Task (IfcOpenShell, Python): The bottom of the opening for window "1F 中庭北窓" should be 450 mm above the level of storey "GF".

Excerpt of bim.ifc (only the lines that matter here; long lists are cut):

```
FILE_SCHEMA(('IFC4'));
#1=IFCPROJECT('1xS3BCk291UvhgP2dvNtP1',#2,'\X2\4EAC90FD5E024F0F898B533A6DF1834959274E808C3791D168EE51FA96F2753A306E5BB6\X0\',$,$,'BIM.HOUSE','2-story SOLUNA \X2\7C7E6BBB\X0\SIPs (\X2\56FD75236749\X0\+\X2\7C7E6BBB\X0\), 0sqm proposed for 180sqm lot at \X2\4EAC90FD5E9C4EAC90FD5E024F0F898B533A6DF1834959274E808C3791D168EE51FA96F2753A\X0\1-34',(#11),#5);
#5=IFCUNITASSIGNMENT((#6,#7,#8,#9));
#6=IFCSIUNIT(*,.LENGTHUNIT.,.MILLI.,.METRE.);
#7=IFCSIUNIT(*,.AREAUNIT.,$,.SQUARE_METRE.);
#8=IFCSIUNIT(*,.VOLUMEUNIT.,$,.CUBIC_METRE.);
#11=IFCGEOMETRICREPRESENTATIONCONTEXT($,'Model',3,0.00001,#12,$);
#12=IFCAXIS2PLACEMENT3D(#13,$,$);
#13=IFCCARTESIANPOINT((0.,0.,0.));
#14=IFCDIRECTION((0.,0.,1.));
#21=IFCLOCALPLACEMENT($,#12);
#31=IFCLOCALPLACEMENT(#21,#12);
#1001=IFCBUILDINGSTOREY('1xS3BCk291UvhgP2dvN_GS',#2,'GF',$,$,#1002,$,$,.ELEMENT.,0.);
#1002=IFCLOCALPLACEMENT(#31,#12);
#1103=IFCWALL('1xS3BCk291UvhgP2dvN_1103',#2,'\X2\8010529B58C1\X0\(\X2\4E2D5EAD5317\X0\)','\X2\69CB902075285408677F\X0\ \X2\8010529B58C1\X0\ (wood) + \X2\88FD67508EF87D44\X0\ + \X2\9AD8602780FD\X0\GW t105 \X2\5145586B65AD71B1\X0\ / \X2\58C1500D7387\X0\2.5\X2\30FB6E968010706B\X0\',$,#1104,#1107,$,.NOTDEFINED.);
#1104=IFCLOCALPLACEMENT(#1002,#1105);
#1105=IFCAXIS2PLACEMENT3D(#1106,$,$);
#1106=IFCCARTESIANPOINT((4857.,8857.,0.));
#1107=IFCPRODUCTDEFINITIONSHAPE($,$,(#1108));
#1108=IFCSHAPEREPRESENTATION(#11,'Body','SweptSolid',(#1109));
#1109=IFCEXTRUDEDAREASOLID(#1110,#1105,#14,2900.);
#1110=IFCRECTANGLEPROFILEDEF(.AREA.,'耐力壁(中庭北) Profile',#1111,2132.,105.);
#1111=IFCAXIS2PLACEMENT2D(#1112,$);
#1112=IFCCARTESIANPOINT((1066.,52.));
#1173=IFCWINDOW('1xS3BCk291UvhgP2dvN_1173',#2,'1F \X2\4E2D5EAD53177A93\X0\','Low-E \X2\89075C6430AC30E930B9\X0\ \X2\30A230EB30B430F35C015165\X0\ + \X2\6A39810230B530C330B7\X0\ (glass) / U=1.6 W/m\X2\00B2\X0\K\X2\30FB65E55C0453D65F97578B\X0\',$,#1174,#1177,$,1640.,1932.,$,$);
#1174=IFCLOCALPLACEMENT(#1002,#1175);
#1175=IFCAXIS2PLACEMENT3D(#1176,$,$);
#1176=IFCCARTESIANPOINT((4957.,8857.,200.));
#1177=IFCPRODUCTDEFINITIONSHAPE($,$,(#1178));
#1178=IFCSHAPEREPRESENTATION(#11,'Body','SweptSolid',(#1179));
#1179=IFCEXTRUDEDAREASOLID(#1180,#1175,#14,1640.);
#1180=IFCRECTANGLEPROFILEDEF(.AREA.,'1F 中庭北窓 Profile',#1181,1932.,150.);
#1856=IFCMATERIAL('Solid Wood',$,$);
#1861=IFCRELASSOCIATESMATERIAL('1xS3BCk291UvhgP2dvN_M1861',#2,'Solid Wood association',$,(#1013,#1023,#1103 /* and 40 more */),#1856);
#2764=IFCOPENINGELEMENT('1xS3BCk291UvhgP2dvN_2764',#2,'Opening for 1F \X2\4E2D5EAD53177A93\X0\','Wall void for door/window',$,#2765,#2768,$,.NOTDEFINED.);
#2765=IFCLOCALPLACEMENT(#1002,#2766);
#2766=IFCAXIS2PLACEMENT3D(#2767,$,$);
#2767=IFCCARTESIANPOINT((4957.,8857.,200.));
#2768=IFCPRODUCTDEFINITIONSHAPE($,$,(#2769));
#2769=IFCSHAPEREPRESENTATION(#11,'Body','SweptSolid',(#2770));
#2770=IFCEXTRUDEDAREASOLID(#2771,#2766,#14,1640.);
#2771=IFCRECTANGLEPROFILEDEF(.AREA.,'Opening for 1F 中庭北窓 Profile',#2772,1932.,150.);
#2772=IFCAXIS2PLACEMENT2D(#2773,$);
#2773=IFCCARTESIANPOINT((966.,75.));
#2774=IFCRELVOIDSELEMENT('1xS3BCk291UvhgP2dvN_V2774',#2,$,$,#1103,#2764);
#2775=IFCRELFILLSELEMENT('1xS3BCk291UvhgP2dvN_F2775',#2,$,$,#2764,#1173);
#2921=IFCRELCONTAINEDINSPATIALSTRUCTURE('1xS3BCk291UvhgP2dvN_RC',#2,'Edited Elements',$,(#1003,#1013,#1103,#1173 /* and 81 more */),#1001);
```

```python
import numpy as np
import ifcopenshell
import ifcopenshell.api.geometry
import ifcopenshell.geom
import ifcopenshell.util.element
import ifcopenshell.util.placement
import ifcopenshell.util.shape
import ifcopenshell.util.unit

model = ifcopenshell.open("bim.ifc")
unit_scale = ifcopenshell.util.unit.calculate_unit_scale(model)

window = model.by_guid("1xS3BCk291UvhgP2dvN_1173")
opening = window.FillsVoids[0].RelatingOpeningElement
storey = ifcopenshell.util.element.get_container(window, ifc_class="IfcBuildingStorey")
level = ifcopenshell.util.placement.get_local_placement(storey.ObjectPlacement)[2, 3]

# The opening's origin need not be at the sill, so measure its lowest point.
shape = ifcopenshell.geom.create_shape(ifcopenshell.geom.settings(), opening)
bottom = ifcopenshell.util.shape.get_shape_bottom_elevation(shape, shape.geometry) / unit_scale
dz = level + 450.0 - bottom

shift = np.array([0.0, 0.0, dz])
# The window is not placed relative to its opening, so move both.
for product in (opening, window):
    matrix = ifcopenshell.util.placement.get_local_placement(product.ObjectPlacement)
    matrix[:3, 3] += shift
    ifcopenshell.api.geometry.edit_object_placement(model, product=product, matrix=matrix, is_si=False)

print(f"moved by {dz * unit_scale:+.3f} m")

model.write("bim-out.ifc")
```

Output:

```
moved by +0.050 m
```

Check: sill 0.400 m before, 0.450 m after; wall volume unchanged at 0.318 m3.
